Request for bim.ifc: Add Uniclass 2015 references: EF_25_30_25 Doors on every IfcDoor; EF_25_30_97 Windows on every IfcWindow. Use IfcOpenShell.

First a look at what the model holds.

```python
import ifcopenshell

model = ifcopenshell.open("bim.ifc")
print(model.schema)
print("classifications:", [c.Name for c in model.by_type("IfcClassification")])
for ifc_class in ("IfcDoor", "IfcRoof", "IfcStair", "IfcWall", "IfcWindow"):
    print(ifc_class, len(model.by_type(ifc_class)))
```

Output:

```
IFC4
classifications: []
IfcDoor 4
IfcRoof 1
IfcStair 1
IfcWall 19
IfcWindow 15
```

```python
import ifcopenshell
import ifcopenshell.api.classification

model = ifcopenshell.open("bim.ifc")

system = ifcopenshell.api.classification.add_classification(model, classification="Uniclass 2015")

codes = {
    "IfcDoor": ("EF_25_30_25", "Doors"),
    "IfcWindow": ("EF_25_30_97", "Windows"),
}
for ifc_class, (code, name) in codes.items():
    products = model.by_type(ifc_class)
    ifcopenshell.api.classification.add_reference(
        model, products=products, classification=system, identification=code, name=name
    )
    print(code, len(products))

model.write("bim-out.ifc")
```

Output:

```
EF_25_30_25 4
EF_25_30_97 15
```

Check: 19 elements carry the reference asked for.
